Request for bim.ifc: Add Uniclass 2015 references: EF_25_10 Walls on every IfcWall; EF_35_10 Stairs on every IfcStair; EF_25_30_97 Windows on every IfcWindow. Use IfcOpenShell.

First a look at what the model holds.

```python
import ifcopenshell

model = ifcopenshell.open("bim.ifc")
print(model.schema)
print("classifications:", [c.Name for c in model.by_type("IfcClassification")])
for ifc_class in ("IfcDoor", "IfcRoof", "IfcStair", "IfcWall", "IfcWindow"):
    print(ifc_class, len(model.by_type(ifc_class)))
```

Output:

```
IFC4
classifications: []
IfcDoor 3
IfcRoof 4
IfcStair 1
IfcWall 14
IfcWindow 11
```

```python
import ifcopenshell
import ifcopenshell.api.classification

model = ifcopenshell.open("bim.ifc")

system = ifcopenshell.api.classification.add_classification(model, classification="Uniclass 2015")

codes = {
    "IfcWall": ("EF_25_10", "Walls"),
    "IfcStair": ("EF_35_10", "Stairs"),
    "IfcWindow": ("EF_25_30_97", "Windows"),
}
for ifc_class, (code, name) in codes.items():
    products = model.by_type(ifc_class)
    ifcopenshell.api.classification.add_reference(
        model, products=products, classification=system, identification=code, name=name
    )
    print(code, len(products))

model.write("bim_v2.ifc")
```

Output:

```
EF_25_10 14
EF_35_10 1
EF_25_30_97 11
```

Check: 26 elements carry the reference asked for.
